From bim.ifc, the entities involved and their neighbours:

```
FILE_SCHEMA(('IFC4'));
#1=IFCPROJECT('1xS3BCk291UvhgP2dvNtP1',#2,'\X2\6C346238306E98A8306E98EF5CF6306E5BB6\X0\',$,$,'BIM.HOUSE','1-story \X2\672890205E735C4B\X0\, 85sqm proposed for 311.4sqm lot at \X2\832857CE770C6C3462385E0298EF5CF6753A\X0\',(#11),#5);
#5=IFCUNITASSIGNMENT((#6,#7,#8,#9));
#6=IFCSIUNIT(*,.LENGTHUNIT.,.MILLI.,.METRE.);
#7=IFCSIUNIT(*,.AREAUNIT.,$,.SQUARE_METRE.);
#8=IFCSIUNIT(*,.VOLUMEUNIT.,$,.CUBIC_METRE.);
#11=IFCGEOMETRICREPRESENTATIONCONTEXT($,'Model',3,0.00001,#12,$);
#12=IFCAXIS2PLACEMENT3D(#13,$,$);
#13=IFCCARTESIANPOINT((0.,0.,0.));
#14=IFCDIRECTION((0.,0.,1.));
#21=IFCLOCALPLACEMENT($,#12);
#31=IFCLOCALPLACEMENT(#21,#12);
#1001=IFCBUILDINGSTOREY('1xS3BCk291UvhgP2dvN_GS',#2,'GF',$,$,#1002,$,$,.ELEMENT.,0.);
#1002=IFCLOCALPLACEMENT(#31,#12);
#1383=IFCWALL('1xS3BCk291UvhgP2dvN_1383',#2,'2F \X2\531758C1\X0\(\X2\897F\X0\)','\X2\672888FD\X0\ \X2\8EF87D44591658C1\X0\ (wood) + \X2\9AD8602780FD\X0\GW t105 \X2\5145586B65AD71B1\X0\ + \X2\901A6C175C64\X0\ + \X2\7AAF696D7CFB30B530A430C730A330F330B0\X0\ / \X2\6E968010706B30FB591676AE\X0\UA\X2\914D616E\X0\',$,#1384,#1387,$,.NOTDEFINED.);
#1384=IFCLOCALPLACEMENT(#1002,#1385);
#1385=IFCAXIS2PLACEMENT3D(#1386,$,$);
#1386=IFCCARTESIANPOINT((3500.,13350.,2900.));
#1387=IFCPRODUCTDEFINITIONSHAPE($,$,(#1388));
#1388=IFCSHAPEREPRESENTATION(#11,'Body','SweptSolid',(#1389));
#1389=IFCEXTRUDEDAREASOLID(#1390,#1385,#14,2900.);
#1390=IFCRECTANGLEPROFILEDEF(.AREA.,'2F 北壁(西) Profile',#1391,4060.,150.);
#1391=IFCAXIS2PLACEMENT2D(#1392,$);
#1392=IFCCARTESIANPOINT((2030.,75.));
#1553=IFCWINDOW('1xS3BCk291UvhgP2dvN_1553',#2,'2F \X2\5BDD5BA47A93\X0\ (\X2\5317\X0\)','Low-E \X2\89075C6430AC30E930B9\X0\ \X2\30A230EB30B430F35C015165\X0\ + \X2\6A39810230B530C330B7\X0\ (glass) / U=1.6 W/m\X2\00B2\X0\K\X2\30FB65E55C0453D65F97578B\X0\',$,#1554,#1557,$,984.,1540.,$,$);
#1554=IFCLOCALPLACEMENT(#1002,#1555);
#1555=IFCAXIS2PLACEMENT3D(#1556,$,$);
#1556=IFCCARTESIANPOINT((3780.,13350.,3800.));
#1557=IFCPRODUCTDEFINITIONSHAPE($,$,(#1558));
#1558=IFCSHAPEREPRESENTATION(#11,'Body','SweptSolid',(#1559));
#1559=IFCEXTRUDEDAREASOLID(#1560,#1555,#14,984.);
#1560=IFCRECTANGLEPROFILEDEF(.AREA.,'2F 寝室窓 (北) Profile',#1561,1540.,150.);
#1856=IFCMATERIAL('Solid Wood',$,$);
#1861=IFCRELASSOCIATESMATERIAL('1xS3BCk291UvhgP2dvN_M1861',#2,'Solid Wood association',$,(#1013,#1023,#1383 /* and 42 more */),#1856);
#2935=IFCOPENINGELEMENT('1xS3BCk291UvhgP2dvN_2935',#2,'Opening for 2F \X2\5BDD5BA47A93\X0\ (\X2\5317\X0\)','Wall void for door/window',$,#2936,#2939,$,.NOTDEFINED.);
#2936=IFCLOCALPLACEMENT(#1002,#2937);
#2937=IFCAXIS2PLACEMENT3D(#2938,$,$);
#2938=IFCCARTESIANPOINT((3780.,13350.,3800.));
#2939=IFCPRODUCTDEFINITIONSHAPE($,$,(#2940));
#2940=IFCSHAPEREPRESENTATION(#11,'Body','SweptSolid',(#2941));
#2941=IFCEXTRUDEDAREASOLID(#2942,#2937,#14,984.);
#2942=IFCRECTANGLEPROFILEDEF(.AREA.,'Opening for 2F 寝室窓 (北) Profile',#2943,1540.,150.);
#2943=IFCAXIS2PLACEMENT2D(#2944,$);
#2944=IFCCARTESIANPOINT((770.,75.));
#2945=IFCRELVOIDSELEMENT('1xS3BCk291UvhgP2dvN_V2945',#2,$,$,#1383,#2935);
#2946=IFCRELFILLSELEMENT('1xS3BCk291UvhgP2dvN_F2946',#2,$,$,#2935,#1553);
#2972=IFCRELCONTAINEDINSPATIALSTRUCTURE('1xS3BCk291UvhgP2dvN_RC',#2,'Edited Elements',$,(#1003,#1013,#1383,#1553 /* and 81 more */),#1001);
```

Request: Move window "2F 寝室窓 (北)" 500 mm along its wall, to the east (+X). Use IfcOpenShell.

```python
import ifcopenshell
import ifcopenshell.api.geometry
import ifcopenshell.util.placement
import ifcopenshell.util.unit

model = ifcopenshell.open("bim.ifc")
unit_scale = ifcopenshell.util.unit.calculate_unit_scale(model)

window = model.by_guid("1xS3BCk291UvhgP2dvN_1553")
opening = window.FillsVoids[0].RelatingOpeningElement
wall = opening.VoidsElements[0].RelatingBuildingElement

wall_matrix = ifcopenshell.util.placement.get_local_placement(wall.ObjectPlacement)
shift = wall_matrix[:3, 0] * 0.5 / unit_scale
before = ifcopenshell.util.placement.get_local_placement(window.ObjectPlacement)[:3, 3].copy()

# The window is not placed relative to its opening, so move both.
for product in (opening, window):
    matrix = ifcopenshell.util.placement.get_local_placement(product.ObjectPlacement)
    matrix[:3, 3] += shift
    ifcopenshell.api.geometry.edit_object_placement(model, product=product, matrix=matrix, is_si=False)

after = ifcopenshell.util.placement.get_local_placement(window.ObjectPlacement)[:3, 3]
print("window moved by", (after - before).round(3) + 0.0)

model.write("bim_edited.ifc")
```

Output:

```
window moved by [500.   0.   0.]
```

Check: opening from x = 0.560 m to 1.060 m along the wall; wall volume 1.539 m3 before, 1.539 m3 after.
